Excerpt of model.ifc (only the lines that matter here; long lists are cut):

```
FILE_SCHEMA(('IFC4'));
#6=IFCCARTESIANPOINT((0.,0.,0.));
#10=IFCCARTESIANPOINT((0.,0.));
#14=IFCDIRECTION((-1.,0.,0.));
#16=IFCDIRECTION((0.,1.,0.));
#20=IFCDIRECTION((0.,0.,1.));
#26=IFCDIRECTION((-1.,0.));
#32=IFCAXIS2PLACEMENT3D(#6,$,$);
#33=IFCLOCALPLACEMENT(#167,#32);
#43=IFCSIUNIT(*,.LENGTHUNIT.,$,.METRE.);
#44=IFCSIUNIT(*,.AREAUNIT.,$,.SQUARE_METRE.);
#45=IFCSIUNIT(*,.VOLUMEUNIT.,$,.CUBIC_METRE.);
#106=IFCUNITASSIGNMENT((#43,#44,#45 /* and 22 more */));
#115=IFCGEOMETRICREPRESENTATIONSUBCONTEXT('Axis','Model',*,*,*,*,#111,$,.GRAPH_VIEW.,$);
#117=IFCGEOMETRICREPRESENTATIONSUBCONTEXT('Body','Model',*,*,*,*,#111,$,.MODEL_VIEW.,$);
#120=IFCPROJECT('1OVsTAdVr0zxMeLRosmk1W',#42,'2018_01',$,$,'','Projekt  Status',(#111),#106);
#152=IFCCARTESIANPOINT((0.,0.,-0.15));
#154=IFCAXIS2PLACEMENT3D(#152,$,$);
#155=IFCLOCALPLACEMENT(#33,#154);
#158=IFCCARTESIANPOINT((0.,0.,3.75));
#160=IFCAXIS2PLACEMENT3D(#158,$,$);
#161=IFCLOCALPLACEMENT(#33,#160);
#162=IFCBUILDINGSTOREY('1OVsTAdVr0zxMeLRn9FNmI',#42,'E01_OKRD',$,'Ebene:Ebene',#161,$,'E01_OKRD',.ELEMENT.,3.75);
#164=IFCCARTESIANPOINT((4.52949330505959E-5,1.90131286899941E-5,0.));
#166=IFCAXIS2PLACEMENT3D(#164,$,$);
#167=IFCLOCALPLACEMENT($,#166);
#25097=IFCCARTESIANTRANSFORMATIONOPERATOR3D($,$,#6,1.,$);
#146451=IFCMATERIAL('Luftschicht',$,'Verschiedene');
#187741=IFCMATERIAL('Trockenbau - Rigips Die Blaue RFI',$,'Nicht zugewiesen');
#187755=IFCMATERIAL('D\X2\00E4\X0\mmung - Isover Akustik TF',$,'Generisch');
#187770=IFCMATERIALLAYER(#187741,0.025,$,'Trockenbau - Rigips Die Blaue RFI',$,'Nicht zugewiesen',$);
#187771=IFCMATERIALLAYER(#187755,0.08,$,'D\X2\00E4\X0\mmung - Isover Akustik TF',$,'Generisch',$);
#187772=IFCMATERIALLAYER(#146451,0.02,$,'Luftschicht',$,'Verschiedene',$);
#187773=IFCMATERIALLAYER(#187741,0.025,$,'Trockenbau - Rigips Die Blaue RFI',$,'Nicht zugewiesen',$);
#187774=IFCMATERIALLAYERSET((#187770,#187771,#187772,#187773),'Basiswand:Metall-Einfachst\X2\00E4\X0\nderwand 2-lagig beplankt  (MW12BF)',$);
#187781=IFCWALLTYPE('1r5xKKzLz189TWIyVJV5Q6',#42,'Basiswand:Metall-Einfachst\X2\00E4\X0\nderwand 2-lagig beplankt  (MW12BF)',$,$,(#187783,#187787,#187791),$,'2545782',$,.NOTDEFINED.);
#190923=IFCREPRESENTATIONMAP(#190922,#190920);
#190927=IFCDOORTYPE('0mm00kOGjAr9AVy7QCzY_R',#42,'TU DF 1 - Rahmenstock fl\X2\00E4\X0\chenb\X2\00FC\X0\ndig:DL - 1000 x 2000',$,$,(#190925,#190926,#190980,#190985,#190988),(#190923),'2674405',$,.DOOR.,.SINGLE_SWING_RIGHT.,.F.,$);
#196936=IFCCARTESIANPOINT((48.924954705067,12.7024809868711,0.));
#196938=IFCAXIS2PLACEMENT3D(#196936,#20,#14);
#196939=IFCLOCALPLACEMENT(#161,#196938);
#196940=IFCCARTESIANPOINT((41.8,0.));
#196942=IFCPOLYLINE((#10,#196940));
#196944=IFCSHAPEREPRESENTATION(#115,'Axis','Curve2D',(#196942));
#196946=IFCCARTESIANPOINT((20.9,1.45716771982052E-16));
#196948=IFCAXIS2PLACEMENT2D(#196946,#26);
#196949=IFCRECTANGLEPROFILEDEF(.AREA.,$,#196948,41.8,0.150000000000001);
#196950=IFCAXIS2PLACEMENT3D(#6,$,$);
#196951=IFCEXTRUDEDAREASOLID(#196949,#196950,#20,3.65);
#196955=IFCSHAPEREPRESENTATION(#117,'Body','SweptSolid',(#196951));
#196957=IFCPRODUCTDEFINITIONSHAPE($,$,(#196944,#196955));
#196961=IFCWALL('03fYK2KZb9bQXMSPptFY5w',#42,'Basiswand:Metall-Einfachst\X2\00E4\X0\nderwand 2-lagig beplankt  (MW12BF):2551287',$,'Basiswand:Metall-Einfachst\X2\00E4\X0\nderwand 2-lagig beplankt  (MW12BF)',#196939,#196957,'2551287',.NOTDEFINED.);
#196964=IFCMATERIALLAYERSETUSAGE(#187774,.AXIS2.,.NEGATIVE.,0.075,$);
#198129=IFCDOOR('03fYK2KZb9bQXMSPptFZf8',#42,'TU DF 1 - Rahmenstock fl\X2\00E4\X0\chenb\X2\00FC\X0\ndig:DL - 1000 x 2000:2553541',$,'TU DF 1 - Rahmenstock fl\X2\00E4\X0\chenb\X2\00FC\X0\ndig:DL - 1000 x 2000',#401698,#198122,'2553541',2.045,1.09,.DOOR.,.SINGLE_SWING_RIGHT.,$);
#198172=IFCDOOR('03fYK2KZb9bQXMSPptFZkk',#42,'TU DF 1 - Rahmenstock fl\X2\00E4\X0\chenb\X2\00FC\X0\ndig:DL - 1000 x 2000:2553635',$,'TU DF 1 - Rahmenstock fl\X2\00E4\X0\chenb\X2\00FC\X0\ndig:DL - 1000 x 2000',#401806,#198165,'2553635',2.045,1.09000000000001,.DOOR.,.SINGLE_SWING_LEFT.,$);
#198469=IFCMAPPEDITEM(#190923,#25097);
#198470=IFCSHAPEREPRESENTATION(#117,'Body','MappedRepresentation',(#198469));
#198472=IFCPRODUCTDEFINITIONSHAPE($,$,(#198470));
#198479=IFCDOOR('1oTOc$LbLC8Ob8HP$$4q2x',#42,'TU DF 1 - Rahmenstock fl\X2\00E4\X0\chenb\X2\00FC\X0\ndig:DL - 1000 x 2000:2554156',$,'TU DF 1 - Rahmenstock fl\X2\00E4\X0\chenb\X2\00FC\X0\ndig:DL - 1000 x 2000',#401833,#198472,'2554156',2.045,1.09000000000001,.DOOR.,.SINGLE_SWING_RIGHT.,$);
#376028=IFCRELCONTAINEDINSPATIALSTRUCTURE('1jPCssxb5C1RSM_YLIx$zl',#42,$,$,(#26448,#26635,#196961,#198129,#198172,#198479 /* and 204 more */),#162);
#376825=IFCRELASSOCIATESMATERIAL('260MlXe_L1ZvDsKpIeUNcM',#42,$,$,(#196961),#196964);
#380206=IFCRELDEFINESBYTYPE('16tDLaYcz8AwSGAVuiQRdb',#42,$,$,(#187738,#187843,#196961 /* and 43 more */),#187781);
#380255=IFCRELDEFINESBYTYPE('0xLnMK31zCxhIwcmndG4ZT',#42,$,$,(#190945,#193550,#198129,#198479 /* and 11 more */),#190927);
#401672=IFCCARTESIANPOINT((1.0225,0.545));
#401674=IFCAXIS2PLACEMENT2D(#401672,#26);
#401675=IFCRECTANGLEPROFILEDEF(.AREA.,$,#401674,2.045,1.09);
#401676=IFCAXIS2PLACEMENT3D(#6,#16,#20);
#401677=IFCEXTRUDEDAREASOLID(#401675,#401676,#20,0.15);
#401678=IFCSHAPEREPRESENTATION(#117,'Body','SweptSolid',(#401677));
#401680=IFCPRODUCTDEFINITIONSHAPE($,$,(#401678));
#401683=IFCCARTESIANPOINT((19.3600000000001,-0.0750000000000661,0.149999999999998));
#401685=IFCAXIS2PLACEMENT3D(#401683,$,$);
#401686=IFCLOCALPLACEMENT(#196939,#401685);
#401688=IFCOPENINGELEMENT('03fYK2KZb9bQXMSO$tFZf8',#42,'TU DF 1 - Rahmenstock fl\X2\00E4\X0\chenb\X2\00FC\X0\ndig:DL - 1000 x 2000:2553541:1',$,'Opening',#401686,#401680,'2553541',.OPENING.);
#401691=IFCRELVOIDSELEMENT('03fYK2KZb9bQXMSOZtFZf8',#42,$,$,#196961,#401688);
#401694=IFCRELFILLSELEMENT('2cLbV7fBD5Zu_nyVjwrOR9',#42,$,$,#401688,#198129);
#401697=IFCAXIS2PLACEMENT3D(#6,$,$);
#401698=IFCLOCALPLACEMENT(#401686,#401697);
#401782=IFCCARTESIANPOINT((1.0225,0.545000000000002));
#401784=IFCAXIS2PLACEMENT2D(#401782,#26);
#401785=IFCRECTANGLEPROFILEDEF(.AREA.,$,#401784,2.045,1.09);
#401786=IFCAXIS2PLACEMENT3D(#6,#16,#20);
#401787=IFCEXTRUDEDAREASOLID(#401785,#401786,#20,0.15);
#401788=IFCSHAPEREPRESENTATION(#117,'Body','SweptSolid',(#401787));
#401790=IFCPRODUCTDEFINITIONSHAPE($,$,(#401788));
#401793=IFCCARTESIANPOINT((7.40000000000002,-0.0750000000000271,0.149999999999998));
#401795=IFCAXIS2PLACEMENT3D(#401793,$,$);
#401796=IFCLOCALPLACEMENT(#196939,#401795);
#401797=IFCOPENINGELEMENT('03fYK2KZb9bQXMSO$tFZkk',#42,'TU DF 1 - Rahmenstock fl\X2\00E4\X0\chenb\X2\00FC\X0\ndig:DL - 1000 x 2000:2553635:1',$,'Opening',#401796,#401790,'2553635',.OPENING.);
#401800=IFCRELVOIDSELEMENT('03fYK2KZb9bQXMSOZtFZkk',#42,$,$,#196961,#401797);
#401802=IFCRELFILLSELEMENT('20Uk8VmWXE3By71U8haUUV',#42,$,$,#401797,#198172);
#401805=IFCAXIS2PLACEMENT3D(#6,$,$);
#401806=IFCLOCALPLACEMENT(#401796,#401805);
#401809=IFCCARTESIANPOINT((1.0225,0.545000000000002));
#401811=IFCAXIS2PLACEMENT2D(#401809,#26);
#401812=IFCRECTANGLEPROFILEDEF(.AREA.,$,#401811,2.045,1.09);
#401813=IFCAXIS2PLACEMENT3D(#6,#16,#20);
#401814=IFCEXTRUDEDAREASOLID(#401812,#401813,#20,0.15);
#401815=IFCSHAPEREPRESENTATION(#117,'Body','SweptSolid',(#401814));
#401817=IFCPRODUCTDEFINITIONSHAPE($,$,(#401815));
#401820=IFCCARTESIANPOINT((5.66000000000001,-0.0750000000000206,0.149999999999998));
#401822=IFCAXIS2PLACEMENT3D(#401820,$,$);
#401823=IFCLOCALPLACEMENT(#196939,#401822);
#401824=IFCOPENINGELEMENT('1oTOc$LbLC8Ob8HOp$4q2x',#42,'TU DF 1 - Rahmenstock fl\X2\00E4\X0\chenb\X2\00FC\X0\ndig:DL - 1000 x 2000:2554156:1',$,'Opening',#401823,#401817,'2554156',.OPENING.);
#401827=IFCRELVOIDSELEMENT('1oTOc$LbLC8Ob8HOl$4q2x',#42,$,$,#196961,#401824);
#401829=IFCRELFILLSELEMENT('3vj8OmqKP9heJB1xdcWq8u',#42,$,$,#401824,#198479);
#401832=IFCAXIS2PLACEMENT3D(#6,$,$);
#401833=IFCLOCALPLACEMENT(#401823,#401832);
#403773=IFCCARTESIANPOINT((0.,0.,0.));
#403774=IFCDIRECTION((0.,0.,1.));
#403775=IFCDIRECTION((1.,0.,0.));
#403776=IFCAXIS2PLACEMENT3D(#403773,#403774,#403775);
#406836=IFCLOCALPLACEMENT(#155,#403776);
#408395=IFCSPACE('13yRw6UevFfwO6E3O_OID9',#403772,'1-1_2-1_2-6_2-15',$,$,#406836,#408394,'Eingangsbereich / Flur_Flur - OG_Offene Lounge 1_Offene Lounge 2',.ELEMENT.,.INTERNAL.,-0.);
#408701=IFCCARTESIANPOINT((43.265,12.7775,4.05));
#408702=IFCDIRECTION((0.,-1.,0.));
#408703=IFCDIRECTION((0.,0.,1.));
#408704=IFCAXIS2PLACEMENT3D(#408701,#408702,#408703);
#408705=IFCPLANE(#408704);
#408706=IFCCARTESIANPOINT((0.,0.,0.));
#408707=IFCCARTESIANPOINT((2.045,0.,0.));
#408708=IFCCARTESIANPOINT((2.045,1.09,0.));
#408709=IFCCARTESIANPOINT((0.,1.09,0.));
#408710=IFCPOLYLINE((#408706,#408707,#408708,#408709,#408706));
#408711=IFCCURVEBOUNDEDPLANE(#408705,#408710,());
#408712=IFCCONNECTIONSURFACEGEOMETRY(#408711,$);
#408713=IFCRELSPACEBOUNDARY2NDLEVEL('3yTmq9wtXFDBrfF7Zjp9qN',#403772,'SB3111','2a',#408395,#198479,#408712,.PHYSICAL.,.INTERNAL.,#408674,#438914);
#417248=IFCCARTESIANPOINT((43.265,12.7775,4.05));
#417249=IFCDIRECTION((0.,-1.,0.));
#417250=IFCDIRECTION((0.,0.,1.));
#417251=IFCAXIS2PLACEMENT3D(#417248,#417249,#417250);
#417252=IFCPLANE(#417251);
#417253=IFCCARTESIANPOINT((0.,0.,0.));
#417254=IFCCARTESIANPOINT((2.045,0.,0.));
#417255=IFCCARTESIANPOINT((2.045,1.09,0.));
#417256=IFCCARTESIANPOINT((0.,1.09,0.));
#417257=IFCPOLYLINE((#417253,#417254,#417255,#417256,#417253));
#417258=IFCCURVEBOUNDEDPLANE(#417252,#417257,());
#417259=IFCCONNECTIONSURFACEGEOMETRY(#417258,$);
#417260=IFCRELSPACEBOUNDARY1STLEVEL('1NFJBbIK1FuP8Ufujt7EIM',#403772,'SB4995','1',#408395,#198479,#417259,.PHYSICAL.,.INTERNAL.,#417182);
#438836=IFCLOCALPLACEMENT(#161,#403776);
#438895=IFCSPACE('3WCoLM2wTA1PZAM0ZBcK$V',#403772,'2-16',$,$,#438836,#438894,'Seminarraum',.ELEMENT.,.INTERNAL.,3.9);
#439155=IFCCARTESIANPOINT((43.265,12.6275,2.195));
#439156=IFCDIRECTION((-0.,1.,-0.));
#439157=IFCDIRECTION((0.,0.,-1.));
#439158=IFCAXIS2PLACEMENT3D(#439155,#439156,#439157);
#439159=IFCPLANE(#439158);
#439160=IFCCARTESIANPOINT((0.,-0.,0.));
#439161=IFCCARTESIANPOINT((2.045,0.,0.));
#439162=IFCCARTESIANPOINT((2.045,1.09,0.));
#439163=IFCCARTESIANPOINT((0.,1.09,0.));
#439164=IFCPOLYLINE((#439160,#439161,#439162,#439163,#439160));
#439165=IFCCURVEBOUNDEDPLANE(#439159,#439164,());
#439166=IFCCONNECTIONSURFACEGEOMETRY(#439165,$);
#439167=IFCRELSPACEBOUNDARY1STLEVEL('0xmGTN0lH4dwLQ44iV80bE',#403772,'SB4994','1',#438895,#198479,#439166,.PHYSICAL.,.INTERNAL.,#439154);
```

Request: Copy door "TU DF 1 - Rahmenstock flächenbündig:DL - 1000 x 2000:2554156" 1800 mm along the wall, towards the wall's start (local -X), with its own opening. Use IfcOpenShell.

```python
import numpy as np
import ifcopenshell
import ifcopenshell.api.feature
import ifcopenshell.api.geometry
import ifcopenshell.api.root
import ifcopenshell.geom
import ifcopenshell.util.element
import ifcopenshell.util.placement
import ifcopenshell.util.shape

model = ifcopenshell.open("model.ifc")
settings = ifcopenshell.geom.settings()


def volume(element):
    """Net volume in cubic metres, openings subtracted."""
    shape = ifcopenshell.geom.create_shape(settings, element)
    return ifcopenshell.util.shape.get_volume(shape.geometry)


def reuse_history(source, copy):
    """copy_class also copies each property set's owner history, people and application; keep the originals."""
    for rel in copy.IsDefinedBy:
        if rel.is_a("IfcRelDefinesByProperties") and (history := rel.RelatingPropertyDefinition.OwnerHistory):
            rel.RelatingPropertyDefinition.OwnerHistory = source.OwnerHistory
            ifcopenshell.util.element.remove_deep2(model, history)


door = model.by_guid("1oTOc$LbLC8Ob8HP$$4q2x")
opening = door.FillsVoids[0].RelatingOpeningElement
wall = opening.VoidsElements[0].RelatingBuildingElement
before = volume(wall)
shift = ifcopenshell.util.placement.get_local_placement(wall.ObjectPlacement)[:3, 0] * -1.8

# copy_class copies the void relationship, type, container and properties, but no geometry.
new_opening = ifcopenshell.api.root.copy_class(model, product=opening)
new_opening.Representation = ifcopenshell.util.element.copy_deep(
    model, opening.Representation, exclude=["IfcGeometricRepresentationContext", "IfcRepresentationMap"]
)
new_opening.Name = "TU DF 1 - Rahmenstock flächenbündig:DL - 1000 x 2000"
new_opening.Tag = None
new_door = ifcopenshell.api.root.copy_class(model, product=door)
new_door.Representation = ifcopenshell.util.element.copy_deep(
    model, door.Representation, exclude=["IfcGeometricRepresentationContext", "IfcRepresentationMap"]
)
new_door.Name = "TU DF 1 - Rahmenstock flächenbündig:DL - 1000 x 2000"
new_door.Tag = None
reuse_history(door, new_door)
ifcopenshell.api.feature.add_filling(model, opening=new_opening, element=new_door)

for old, new in ((opening, new_opening), (door, new_door)):
    matrix = ifcopenshell.util.placement.get_local_placement(old.ObjectPlacement)
    matrix[:3, 3] += shift
    ifcopenshell.api.geometry.edit_object_placement(model, product=new, matrix=matrix, is_si=False)

# The copied space boundaries still share their surfaces with the original.
for rel in new_door.ProvidesBoundaries:
    if rel.ConnectionGeometry:
        rel.ConnectionGeometry = ifcopenshell.util.element.copy_deep(model, rel.ConnectionGeometry)

# Space boundary surfaces are stored in each space's coordinates; move them too.
for rel in new_door.ProvidesBoundaries:
    if not rel.ConnectionGeometry:
        continue
    surface = rel.ConnectionGeometry.SurfaceOnRelatingElement.BasisSurface
    space_matrix = ifcopenshell.util.placement.get_local_placement(rel.RelatingSpace.ObjectPlacement)
    point = np.array(surface.Position.Location.Coordinates) + space_matrix[:3, :3].T @ shift
    surface.Position = model.createIfcAxis2Placement3D(
        model.createIfcCartesianPoint(point.tolist()), surface.Position.Axis, surface.Position.RefDirection
    )

after = volume(wall)

print(f"wall volume {before:.3f} -> {after:.3f} m3")

model.write("model_edited.ifc")
```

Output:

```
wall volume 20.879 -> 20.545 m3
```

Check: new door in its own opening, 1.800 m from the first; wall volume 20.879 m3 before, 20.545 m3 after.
